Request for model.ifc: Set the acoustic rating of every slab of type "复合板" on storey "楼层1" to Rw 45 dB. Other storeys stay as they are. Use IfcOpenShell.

First a look at what the model holds.

```python
import ifcopenshell
import ifcopenshell.util.element

model = ifcopenshell.open("model.ifc")
print(model.schema)
storey = next(s for s in model.by_type("IfcBuildingStorey") if s.Name == "楼层1")
slabs = [e for e in ifcopenshell.util.element.get_decomposition(storey) if e.is_a("IfcSlab")]
seen = {}
for e in slabs:
    element_type = ifcopenshell.util.element.get_type(e)
    key = (element_type.Name if element_type != e and element_type else None, ifcopenshell.util.element.get_pset(e, "Pset_SlabCommon", "AcousticRating"))
    seen[key] = seen.get(key, 0) + 1
for (name, value), count in sorted(seen.items(), key=str):
    print(count, "x", name, "|", value)
```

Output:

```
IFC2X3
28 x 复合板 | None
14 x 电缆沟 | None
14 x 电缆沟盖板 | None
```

```python
import ifcopenshell
import ifcopenshell.api.pset
import ifcopenshell.util.element

model = ifcopenshell.open("model.ifc")

storey = next(s for s in model.by_type("IfcBuildingStorey") if s.Name == "楼层1")
slabs = [e for e in ifcopenshell.util.element.get_decomposition(storey) if e.is_a("IfcSlab")]

count = 0
for e in slabs:
    element_type = ifcopenshell.util.element.get_type(e)
    if element_type in (None, e) or element_type.Name != "复合板":
        continue
    # add_pset returns the element's existing set when there is one.
    pset = ifcopenshell.api.pset.add_pset(model, product=e, name="Pset_SlabCommon")
    ifcopenshell.api.pset.edit_pset(model, pset=pset, properties={"AcousticRating": "Rw 45 dB"})
    count += 1

print(count, "slabs updated")

model.write("model_updated.ifc")
```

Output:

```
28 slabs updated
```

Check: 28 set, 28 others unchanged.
